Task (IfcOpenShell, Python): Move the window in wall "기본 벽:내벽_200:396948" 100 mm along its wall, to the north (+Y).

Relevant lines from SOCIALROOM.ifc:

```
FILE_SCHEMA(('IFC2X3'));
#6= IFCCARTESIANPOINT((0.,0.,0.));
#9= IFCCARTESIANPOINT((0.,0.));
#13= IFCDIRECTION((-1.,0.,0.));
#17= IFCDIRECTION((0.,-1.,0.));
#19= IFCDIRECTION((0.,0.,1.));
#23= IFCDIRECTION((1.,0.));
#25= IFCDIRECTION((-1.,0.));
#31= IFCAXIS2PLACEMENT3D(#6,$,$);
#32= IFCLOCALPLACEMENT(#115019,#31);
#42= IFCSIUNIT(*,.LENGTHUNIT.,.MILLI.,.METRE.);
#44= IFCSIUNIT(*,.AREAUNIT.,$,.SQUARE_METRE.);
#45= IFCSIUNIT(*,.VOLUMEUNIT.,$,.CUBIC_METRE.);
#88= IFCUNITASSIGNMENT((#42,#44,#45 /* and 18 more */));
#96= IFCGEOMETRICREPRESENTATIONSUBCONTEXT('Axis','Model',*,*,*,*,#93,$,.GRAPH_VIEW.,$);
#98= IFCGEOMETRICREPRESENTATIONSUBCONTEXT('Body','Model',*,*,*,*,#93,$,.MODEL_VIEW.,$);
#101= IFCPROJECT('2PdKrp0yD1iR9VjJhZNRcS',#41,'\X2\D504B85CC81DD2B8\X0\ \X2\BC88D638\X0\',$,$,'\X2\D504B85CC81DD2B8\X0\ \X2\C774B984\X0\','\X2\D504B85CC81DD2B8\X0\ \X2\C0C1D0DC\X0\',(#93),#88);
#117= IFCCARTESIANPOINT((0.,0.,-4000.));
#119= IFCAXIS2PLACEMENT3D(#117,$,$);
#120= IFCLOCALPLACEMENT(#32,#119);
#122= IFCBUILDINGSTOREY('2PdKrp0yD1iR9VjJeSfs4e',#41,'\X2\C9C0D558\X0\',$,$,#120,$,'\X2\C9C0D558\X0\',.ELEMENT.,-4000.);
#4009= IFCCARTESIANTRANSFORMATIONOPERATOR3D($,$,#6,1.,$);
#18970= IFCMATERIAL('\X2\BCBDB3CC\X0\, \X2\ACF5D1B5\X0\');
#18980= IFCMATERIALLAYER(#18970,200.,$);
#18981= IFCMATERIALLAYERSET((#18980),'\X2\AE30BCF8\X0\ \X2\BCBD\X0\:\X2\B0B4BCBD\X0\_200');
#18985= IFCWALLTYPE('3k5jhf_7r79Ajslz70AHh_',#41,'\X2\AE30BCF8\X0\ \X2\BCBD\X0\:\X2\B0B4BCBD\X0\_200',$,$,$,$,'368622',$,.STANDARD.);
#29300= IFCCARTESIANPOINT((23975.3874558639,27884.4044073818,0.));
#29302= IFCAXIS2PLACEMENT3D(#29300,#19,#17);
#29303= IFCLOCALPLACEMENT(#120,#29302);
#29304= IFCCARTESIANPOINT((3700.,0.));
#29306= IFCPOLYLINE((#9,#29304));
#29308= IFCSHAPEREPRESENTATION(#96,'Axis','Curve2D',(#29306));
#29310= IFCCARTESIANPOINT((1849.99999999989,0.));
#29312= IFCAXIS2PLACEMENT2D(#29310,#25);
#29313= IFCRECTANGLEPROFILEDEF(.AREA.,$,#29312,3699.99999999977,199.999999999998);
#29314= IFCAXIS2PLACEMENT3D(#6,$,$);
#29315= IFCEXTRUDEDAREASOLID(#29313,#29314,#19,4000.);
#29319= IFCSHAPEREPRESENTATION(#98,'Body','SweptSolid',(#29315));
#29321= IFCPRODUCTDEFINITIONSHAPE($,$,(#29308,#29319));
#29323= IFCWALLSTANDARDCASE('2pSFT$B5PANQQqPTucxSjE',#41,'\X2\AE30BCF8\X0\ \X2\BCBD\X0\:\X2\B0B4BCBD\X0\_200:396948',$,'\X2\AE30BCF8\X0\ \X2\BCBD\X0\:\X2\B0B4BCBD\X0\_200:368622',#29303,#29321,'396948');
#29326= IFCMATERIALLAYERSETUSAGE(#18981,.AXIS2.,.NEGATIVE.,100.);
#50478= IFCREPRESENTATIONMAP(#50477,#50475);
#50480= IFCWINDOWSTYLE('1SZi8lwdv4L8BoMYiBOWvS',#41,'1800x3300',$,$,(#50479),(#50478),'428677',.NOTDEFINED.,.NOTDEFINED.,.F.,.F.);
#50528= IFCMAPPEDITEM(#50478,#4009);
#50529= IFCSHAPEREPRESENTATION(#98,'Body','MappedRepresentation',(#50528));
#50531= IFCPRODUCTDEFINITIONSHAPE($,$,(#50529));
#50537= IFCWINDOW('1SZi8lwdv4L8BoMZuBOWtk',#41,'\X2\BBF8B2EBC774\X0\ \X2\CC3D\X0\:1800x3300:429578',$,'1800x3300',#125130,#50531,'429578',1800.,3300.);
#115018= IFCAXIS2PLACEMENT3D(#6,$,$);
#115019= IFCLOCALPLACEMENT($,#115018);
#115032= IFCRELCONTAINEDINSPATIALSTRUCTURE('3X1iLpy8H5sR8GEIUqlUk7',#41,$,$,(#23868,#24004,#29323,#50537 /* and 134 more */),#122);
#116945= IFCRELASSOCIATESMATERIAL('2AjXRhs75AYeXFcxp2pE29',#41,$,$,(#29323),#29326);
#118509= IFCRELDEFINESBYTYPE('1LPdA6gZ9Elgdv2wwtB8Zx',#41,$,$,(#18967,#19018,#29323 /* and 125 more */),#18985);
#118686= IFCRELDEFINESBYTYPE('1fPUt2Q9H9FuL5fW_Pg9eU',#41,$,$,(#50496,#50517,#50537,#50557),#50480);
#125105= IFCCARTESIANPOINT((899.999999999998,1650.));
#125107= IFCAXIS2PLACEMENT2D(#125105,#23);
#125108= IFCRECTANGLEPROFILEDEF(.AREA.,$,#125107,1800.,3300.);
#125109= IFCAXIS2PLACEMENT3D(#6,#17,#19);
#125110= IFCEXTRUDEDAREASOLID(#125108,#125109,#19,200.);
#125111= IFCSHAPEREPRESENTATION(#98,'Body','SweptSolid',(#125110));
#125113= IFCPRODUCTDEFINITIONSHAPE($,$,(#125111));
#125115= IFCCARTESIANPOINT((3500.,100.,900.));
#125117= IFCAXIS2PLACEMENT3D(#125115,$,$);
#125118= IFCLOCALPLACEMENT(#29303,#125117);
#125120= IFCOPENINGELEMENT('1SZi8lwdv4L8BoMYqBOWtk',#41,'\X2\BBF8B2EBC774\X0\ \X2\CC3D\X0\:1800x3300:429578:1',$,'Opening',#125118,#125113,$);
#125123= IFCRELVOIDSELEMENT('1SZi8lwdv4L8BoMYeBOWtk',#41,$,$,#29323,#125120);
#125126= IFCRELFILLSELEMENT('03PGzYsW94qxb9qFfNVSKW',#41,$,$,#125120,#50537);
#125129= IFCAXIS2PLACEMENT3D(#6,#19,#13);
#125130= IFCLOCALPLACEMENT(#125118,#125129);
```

```python
import ifcopenshell
import ifcopenshell.api.geometry
import ifcopenshell.util.placement
import ifcopenshell.util.unit

model = ifcopenshell.open("SOCIALROOM.ifc")
unit_scale = ifcopenshell.util.unit.calculate_unit_scale(model)

window = model.by_guid("1SZi8lwdv4L8BoMZuBOWtk")
opening = window.FillsVoids[0].RelatingOpeningElement
wall = opening.VoidsElements[0].RelatingBuildingElement

wall_matrix = ifcopenshell.util.placement.get_local_placement(wall.ObjectPlacement)
shift = wall_matrix[:3, 0] * -0.1 / unit_scale
before = ifcopenshell.util.placement.get_local_placement(window.ObjectPlacement)[:3, 3].copy()

# The window is placed relative to its opening, so it follows when the opening moves.
matrix = ifcopenshell.util.placement.get_local_placement(opening.ObjectPlacement)
matrix[:3, 3] += shift
ifcopenshell.api.geometry.edit_object_placement(
    model, product=opening, matrix=matrix, is_si=False, should_transform_children=True
)

after = ifcopenshell.util.placement.get_local_placement(window.ObjectPlacement)[:3, 3]
print("window moved by", (after - before).round(3) + 0.0)

model.write("SOCIALROOM_updated.ifc")
```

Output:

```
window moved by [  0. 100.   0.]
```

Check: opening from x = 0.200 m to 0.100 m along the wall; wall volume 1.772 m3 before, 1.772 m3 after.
